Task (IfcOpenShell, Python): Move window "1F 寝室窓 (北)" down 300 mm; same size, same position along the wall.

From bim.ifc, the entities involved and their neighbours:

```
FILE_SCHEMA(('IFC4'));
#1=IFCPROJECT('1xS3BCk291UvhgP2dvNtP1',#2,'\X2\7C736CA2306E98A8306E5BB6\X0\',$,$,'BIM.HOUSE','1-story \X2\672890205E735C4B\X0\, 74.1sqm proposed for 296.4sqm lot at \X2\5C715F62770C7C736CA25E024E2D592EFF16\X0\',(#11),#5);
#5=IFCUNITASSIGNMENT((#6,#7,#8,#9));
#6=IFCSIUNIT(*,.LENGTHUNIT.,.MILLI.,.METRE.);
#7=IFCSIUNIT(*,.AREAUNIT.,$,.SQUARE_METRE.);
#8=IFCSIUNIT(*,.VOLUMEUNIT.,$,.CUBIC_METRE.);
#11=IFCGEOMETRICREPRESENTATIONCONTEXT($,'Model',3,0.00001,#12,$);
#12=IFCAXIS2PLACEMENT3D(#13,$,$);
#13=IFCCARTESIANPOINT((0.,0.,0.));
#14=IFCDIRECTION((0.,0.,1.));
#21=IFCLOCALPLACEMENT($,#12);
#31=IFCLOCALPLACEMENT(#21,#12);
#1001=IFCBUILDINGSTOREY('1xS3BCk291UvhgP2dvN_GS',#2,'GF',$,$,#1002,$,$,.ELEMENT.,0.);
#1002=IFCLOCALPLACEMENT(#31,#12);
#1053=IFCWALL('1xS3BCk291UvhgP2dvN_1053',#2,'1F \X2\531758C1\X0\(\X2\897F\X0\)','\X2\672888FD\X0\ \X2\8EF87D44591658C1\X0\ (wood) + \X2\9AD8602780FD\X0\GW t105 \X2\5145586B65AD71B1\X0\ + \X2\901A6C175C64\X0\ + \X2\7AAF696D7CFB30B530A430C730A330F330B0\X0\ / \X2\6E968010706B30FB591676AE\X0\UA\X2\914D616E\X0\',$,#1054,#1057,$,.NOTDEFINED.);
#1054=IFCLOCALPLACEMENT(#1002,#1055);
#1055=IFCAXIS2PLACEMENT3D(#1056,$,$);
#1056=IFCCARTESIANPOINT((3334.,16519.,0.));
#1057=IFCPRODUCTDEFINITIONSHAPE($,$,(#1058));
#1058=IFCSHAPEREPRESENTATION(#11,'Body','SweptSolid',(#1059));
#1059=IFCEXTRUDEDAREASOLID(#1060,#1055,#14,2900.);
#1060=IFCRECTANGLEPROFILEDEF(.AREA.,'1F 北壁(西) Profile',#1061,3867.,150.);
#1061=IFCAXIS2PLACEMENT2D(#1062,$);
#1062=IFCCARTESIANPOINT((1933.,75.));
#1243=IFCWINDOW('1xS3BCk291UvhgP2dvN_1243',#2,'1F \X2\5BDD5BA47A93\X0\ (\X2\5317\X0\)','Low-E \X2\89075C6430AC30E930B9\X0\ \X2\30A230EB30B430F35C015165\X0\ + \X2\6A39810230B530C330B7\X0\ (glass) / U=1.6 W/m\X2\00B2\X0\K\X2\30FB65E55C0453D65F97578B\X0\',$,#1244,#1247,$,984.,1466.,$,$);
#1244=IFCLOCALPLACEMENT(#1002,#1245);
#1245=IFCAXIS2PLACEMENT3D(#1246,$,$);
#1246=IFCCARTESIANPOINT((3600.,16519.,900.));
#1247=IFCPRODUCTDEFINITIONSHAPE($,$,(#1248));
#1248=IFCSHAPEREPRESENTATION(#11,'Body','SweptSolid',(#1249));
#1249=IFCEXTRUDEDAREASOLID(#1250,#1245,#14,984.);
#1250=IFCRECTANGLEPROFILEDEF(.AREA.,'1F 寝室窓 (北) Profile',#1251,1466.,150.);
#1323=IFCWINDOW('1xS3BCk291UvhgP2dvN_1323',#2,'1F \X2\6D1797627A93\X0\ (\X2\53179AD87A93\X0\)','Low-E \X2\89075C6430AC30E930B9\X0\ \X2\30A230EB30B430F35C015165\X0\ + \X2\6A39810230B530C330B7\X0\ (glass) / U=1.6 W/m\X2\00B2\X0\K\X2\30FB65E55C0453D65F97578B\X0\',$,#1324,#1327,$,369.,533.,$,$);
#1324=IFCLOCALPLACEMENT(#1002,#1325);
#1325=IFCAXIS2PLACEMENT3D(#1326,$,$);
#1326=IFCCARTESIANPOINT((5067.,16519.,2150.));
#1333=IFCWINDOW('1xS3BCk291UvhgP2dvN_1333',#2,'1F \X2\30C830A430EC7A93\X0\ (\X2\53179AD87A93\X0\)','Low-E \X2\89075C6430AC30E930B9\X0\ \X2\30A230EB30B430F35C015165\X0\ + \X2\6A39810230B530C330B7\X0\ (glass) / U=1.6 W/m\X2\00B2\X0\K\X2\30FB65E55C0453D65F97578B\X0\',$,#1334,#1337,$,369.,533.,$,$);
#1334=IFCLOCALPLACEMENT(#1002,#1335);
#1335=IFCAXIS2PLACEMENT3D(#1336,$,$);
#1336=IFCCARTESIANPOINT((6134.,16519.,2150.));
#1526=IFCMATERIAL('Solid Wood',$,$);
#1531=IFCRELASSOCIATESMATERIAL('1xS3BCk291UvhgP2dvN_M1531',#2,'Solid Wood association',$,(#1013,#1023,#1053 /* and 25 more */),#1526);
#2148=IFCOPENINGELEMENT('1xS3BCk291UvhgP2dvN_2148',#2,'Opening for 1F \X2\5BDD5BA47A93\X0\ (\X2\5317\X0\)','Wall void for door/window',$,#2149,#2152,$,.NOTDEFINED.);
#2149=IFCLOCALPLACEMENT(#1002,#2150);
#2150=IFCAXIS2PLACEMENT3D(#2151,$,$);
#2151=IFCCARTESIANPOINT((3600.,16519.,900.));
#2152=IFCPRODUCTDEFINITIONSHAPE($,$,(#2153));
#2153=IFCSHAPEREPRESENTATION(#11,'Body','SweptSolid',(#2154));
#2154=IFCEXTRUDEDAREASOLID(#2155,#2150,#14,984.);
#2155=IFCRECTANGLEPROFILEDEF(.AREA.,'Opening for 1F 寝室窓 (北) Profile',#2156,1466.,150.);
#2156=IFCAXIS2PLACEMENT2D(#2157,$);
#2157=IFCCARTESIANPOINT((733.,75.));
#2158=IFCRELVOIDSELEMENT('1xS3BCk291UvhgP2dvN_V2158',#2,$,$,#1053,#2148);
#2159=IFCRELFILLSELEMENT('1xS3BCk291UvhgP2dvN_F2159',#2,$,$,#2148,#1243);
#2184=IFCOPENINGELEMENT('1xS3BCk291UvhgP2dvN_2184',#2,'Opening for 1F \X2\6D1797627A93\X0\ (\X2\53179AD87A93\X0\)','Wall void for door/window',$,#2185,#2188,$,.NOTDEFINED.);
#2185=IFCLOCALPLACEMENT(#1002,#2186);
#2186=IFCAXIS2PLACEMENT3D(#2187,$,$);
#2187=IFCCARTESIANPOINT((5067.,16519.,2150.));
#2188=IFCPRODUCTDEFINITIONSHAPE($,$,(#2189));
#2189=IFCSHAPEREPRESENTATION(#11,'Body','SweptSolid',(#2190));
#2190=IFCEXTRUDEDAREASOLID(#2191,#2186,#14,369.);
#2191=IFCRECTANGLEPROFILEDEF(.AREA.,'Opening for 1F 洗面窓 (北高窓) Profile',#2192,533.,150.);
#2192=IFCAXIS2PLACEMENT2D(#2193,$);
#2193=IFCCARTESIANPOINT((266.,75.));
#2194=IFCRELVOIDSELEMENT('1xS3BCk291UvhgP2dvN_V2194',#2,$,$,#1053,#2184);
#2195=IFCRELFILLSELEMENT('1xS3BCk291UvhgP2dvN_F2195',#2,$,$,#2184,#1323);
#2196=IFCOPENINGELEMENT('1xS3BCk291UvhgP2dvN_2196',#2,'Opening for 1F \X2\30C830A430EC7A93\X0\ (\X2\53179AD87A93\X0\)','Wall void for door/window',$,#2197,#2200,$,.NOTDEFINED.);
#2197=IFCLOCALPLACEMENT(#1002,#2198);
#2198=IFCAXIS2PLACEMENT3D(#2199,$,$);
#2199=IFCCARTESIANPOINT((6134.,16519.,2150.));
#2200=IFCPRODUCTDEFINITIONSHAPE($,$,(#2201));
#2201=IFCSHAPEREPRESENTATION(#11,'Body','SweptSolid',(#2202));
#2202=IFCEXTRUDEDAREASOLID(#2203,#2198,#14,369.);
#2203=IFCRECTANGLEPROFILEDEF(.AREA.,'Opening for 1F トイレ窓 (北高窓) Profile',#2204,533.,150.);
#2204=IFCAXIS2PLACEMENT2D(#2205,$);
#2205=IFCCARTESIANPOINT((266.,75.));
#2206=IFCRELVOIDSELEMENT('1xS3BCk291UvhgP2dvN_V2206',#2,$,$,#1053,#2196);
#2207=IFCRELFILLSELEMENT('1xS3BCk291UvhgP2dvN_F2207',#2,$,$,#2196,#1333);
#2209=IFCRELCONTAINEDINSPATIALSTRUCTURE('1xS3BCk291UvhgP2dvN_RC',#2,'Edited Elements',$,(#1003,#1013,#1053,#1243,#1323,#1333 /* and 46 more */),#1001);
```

```python
import numpy as np
import ifcopenshell
import ifcopenshell.api.geometry
import ifcopenshell.util.placement
import ifcopenshell.util.unit

model = ifcopenshell.open("bim.ifc")
unit_scale = ifcopenshell.util.unit.calculate_unit_scale(model)

window = model.by_id(1243)
opening = window.FillsVoids[0].RelatingOpeningElement
dz = -300.0

shift = np.array([0.0, 0.0, dz])
# The window is not placed relative to its opening, so move both.
for product in (opening, window):
    matrix = ifcopenshell.util.placement.get_local_placement(product.ObjectPlacement)
    matrix[:3, 3] += shift
    ifcopenshell.api.geometry.edit_object_placement(model, product=product, matrix=matrix, is_si=False)

print(f"moved by {dz * unit_scale:+.3f} m")

model.write("bim_edited.ifc")
```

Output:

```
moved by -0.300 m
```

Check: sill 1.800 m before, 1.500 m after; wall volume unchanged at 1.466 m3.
